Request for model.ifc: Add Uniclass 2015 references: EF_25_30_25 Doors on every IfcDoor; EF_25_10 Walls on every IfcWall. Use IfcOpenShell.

First a look at what the model holds.

```python
import ifcopenshell

model = ifcopenshell.open("model.ifc")
print(model.schema)
print("classifications:", [c.Name for c in model.by_type("IfcClassification")])
for ifc_class in ("IfcDoor", "IfcRoof", "IfcStair", "IfcWall", "IfcWindow"):
    print(ifc_class, len(model.by_type(ifc_class)))
```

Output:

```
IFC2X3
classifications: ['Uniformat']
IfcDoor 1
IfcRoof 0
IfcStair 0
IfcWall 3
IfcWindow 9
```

```python
import ifcopenshell
import ifcopenshell.api.classification

model = ifcopenshell.open("model.ifc")

# IFC2X3 requires Source and Edition and has no link from the project to the system.
system = model.create_entity("IfcClassification", Source="NBS", Edition="2015", Name="Uniclass 2015")

codes = {
    "IfcDoor": ("EF_25_30_25", "Doors"),
    "IfcWall": ("EF_25_10", "Walls"),
}
for ifc_class, (code, name) in codes.items():
    products = model.by_type(ifc_class)
    ifcopenshell.api.classification.add_reference(
        model, products=products, classification=system, identification=code, name=name
    )
    print(code, len(products))

model.write("model_rev.ifc")
```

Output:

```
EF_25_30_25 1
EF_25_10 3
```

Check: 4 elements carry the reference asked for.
